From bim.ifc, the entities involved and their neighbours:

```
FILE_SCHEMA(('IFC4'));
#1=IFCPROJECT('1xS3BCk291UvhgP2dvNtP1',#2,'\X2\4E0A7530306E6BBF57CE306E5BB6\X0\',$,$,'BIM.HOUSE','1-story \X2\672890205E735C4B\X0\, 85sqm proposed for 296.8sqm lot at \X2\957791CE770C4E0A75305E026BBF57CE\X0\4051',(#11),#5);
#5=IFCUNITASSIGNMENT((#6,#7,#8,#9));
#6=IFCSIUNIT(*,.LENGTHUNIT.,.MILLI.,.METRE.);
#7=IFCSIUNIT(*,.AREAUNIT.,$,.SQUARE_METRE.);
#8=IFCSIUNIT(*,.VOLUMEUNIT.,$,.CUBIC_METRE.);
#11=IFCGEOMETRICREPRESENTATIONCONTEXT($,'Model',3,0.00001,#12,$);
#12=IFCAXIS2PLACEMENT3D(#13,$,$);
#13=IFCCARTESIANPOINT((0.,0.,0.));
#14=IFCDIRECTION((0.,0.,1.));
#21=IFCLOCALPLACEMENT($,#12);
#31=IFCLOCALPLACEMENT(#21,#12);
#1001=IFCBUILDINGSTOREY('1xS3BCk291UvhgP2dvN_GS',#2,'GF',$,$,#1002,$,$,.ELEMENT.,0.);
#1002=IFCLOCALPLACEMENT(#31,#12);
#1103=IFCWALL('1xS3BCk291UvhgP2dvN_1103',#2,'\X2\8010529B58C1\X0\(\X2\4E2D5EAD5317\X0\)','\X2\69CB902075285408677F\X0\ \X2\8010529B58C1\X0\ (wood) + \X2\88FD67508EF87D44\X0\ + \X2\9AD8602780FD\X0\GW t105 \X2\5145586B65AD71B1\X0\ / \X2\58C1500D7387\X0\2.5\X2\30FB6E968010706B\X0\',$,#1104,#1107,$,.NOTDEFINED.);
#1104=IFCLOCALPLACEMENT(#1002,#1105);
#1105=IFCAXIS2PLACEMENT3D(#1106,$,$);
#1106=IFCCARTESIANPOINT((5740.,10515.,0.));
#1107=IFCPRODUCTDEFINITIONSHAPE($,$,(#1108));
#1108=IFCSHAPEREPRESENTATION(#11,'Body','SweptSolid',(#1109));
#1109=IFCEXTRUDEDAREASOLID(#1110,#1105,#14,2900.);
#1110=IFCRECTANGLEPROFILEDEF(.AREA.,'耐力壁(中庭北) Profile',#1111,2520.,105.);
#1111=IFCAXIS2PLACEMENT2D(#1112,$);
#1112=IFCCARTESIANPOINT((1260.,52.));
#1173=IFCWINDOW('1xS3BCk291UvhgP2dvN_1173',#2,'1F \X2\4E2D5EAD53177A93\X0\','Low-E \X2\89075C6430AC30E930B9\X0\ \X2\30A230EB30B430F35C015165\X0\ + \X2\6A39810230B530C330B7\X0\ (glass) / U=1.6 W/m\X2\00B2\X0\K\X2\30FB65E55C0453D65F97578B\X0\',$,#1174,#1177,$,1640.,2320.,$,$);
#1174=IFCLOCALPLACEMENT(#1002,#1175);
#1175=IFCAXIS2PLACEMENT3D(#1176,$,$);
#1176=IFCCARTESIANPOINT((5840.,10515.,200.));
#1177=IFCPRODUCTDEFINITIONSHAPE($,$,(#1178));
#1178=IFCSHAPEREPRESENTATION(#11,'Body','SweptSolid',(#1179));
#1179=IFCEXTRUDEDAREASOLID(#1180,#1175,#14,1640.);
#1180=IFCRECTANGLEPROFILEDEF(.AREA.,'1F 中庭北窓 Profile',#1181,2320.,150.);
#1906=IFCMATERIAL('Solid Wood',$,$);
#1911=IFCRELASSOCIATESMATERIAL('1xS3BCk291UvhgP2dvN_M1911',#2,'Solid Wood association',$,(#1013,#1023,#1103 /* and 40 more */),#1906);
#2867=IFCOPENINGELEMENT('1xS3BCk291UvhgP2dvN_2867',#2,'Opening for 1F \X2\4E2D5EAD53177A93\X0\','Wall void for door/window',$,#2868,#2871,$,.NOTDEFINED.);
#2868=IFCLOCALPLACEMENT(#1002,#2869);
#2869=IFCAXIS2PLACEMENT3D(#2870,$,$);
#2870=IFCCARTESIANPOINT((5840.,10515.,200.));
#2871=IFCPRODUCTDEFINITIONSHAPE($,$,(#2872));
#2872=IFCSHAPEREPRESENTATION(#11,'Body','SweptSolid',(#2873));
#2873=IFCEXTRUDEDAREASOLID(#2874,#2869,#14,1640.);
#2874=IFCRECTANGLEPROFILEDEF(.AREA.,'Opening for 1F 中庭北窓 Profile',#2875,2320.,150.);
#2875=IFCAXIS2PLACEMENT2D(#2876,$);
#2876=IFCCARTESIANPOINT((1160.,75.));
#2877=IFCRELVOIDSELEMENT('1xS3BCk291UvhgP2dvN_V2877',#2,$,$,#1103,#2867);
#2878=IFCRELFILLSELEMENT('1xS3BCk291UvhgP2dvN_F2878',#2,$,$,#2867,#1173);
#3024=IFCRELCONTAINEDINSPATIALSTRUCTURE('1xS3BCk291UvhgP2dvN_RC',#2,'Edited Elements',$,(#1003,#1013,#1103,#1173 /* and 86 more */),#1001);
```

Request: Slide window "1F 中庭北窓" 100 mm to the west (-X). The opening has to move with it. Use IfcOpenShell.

```python
import ifcopenshell
import ifcopenshell.api.geometry
import ifcopenshell.util.placement
import ifcopenshell.util.unit

model = ifcopenshell.open("bim.ifc")
unit_scale = ifcopenshell.util.unit.calculate_unit_scale(model)

window = model.by_guid("1xS3BCk291UvhgP2dvN_1173")
opening = window.FillsVoids[0].RelatingOpeningElement
wall = opening.VoidsElements[0].RelatingBuildingElement

wall_matrix = ifcopenshell.util.placement.get_local_placement(wall.ObjectPlacement)
shift = wall_matrix[:3, 0] * -0.1 / unit_scale
before = ifcopenshell.util.placement.get_local_placement(window.ObjectPlacement)[:3, 3].copy()

# The window is not placed relative to its opening, so move both.
for product in (opening, window):
    matrix = ifcopenshell.util.placement.get_local_placement(product.ObjectPlacement)
    matrix[:3, 3] += shift
    ifcopenshell.api.geometry.edit_object_placement(model, product=product, matrix=matrix, is_si=False)

after = ifcopenshell.util.placement.get_local_placement(window.ObjectPlacement)[:3, 3]
print("window moved by", (after - before).round(3) + 0.0)

model.write("bim_rev.ifc")
```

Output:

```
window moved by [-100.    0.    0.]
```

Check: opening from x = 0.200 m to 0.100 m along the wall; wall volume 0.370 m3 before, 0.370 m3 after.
